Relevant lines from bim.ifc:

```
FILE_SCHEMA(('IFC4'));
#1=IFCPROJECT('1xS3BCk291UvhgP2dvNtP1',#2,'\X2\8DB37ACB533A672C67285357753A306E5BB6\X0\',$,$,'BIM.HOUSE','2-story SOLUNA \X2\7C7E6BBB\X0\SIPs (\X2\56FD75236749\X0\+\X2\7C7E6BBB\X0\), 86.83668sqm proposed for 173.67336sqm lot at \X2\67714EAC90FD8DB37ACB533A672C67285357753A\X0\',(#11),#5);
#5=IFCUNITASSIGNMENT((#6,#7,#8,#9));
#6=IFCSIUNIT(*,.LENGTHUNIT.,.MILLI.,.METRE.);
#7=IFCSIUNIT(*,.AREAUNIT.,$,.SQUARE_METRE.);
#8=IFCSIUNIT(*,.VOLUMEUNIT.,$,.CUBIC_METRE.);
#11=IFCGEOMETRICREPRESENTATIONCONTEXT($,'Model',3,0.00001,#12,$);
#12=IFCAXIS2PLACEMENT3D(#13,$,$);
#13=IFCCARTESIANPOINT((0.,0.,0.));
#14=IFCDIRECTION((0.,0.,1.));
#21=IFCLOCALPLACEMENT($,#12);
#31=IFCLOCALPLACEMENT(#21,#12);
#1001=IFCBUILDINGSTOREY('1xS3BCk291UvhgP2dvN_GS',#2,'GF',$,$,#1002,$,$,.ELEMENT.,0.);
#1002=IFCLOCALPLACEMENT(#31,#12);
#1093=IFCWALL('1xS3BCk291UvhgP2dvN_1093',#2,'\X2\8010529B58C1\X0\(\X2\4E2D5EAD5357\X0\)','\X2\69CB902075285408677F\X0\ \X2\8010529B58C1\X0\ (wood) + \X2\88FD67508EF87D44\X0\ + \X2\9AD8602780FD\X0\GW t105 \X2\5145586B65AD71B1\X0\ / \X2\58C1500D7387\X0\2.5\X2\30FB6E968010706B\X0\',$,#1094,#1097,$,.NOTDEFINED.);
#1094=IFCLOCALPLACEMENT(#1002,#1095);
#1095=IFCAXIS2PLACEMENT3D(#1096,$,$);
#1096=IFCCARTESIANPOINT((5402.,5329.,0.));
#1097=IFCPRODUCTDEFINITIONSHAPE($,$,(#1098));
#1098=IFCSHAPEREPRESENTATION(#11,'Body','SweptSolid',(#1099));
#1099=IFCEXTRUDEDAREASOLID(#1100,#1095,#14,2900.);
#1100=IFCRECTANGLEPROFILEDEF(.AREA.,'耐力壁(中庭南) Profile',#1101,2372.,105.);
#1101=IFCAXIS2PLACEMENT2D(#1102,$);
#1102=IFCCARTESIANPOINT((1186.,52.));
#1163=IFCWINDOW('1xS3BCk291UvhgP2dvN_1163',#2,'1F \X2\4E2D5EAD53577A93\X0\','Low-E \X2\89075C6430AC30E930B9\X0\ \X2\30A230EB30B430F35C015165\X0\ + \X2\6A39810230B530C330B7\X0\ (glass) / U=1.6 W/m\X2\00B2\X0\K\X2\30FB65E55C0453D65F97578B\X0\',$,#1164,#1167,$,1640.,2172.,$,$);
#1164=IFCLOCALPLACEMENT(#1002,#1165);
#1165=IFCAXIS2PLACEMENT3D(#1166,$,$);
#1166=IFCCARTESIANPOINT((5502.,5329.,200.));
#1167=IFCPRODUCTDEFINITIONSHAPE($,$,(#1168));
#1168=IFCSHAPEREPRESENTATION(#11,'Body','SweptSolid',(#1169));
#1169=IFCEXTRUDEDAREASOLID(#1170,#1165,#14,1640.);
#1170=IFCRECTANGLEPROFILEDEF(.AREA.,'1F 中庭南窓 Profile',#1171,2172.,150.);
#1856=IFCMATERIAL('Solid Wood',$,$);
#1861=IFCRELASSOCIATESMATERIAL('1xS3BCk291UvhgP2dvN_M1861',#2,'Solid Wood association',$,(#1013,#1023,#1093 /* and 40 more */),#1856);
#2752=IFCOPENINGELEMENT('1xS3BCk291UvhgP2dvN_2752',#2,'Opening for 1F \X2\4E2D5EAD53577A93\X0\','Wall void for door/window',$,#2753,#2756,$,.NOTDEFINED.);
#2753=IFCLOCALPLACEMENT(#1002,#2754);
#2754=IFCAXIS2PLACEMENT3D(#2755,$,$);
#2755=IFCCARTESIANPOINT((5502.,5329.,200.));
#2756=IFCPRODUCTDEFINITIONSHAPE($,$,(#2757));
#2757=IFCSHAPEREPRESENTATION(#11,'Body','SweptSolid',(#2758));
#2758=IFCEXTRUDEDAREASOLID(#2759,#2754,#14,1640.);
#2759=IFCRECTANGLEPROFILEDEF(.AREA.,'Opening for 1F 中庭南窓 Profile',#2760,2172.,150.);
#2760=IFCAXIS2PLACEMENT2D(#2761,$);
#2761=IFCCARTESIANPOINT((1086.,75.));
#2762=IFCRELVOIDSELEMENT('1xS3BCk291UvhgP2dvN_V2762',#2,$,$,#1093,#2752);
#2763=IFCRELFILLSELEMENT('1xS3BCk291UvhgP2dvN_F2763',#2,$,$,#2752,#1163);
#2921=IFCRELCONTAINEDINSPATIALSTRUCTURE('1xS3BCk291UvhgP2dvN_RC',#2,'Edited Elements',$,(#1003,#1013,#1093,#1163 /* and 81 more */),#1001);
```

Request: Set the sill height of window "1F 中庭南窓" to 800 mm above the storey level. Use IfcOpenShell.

```python
import numpy as np
import ifcopenshell
import ifcopenshell.api.geometry
import ifcopenshell.geom
import ifcopenshell.util.element
import ifcopenshell.util.placement
import ifcopenshell.util.shape
import ifcopenshell.util.unit

model = ifcopenshell.open("bim.ifc")
unit_scale = ifcopenshell.util.unit.calculate_unit_scale(model)

window = model.by_guid("1xS3BCk291UvhgP2dvN_1163")
opening = window.FillsVoids[0].RelatingOpeningElement
storey = ifcopenshell.util.element.get_container(window, ifc_class="IfcBuildingStorey")
level = ifcopenshell.util.placement.get_local_placement(storey.ObjectPlacement)[2, 3]

# The opening's origin need not be at the sill, so measure its lowest point.
shape = ifcopenshell.geom.create_shape(ifcopenshell.geom.settings(), opening)
bottom = ifcopenshell.util.shape.get_shape_bottom_elevation(shape, shape.geometry) / unit_scale
dz = level + 0.8 / unit_scale - bottom

shift = np.array([0.0, 0.0, dz])
# The window is not placed relative to its opening, so move both.
for product in (opening, window):
    matrix = ifcopenshell.util.placement.get_local_placement(product.ObjectPlacement)
    matrix[:3, 3] += shift
    ifcopenshell.api.geometry.edit_object_placement(model, product=product, matrix=matrix, is_si=False)

print(f"moved by {dz * unit_scale:+.3f} m")

model.write("bim_updated.ifc")
```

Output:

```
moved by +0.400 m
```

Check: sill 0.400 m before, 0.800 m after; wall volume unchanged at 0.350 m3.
